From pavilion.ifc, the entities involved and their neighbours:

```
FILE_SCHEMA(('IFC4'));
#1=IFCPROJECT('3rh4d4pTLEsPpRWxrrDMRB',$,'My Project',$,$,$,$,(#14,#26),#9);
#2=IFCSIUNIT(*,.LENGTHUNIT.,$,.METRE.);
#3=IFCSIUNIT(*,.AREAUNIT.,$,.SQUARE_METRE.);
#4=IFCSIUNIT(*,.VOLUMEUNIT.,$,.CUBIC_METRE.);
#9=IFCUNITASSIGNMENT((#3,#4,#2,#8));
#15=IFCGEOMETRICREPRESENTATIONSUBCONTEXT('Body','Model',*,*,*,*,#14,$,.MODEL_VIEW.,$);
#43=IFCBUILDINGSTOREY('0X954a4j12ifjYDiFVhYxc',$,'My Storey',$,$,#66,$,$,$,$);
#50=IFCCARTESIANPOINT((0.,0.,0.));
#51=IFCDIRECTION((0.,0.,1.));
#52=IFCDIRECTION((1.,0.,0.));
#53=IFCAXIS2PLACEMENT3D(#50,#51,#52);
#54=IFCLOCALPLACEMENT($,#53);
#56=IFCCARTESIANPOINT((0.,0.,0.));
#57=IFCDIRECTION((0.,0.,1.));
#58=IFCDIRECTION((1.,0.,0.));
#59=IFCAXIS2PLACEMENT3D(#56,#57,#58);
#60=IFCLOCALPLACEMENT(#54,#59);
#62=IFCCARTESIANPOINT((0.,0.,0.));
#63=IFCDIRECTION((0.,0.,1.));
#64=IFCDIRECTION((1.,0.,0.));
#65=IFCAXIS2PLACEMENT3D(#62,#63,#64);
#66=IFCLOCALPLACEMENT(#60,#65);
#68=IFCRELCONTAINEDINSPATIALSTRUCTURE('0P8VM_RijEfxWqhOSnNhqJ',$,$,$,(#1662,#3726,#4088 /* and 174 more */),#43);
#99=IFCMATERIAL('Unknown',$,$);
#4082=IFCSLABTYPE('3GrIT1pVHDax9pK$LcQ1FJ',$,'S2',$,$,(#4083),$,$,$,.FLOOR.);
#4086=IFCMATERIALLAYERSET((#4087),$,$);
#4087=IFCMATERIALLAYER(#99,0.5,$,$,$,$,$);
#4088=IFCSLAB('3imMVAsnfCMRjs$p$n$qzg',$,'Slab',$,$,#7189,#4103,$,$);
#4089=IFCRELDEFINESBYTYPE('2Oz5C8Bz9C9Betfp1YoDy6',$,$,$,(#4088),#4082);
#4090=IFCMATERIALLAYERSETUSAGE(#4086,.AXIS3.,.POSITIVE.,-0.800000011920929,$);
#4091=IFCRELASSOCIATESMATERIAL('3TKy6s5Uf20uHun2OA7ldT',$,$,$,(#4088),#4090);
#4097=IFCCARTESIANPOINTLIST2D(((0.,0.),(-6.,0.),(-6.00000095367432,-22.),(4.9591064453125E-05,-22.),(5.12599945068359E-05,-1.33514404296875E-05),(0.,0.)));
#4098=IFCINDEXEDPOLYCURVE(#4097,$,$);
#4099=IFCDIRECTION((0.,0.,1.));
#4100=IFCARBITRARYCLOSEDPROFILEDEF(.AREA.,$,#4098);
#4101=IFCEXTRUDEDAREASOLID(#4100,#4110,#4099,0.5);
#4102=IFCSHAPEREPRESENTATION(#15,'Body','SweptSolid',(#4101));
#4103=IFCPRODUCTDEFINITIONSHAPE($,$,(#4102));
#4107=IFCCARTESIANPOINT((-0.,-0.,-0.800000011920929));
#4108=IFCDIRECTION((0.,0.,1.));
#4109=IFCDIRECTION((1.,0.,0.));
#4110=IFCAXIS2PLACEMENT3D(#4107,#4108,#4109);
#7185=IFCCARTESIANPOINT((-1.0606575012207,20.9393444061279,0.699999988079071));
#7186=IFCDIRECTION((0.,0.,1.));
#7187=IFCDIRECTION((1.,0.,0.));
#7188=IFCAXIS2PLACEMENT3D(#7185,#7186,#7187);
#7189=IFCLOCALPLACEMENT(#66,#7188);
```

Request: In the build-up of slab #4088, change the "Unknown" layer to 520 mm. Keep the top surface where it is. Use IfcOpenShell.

```python
import ifcopenshell
import ifcopenshell.util.element
import ifcopenshell.util.representation

model = ifcopenshell.open("pavilion.ifc")

layer_set = model.by_id(4086)
layer = next(l for l in layer_set.MaterialLayers if l.Material and l.Material.Name == "Unknown")
change = 0.52 - layer.LayerThickness
layer.LayerThickness += change

# Geometry does not follow the layer set by itself.
slabs = [e for e in ifcopenshell.util.element.get_elements_by_material(model, layer_set) if e.is_a("IfcSlab")]
for slab in sorted(slabs, key=lambda e: e.id()):
    body = ifcopenshell.util.representation.get_representation(slab, "Model", "Body")
    solid = body.Items[0]
    old_depth = solid.Depth
    solid.Depth += change
    # Extruded upwards: lower the start of the extrusion so the top stays.
    x, y, z = solid.Position.Location.Coordinates
    solid.Position.Location = model.createIfcCartesianPoint((x, y, z - change))
    print(slab.id(), f"{old_depth:g} -> {solid.Depth:g}")

# The layers are counted up from the underside, which has moved.
for usage in {ifcopenshell.util.element.get_material(slab) for slab in slabs}:
    usage.OffsetFromReferenceLine -= change

model.write("pavilion-out.ifc")
```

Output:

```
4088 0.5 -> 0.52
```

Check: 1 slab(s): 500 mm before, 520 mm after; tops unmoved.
